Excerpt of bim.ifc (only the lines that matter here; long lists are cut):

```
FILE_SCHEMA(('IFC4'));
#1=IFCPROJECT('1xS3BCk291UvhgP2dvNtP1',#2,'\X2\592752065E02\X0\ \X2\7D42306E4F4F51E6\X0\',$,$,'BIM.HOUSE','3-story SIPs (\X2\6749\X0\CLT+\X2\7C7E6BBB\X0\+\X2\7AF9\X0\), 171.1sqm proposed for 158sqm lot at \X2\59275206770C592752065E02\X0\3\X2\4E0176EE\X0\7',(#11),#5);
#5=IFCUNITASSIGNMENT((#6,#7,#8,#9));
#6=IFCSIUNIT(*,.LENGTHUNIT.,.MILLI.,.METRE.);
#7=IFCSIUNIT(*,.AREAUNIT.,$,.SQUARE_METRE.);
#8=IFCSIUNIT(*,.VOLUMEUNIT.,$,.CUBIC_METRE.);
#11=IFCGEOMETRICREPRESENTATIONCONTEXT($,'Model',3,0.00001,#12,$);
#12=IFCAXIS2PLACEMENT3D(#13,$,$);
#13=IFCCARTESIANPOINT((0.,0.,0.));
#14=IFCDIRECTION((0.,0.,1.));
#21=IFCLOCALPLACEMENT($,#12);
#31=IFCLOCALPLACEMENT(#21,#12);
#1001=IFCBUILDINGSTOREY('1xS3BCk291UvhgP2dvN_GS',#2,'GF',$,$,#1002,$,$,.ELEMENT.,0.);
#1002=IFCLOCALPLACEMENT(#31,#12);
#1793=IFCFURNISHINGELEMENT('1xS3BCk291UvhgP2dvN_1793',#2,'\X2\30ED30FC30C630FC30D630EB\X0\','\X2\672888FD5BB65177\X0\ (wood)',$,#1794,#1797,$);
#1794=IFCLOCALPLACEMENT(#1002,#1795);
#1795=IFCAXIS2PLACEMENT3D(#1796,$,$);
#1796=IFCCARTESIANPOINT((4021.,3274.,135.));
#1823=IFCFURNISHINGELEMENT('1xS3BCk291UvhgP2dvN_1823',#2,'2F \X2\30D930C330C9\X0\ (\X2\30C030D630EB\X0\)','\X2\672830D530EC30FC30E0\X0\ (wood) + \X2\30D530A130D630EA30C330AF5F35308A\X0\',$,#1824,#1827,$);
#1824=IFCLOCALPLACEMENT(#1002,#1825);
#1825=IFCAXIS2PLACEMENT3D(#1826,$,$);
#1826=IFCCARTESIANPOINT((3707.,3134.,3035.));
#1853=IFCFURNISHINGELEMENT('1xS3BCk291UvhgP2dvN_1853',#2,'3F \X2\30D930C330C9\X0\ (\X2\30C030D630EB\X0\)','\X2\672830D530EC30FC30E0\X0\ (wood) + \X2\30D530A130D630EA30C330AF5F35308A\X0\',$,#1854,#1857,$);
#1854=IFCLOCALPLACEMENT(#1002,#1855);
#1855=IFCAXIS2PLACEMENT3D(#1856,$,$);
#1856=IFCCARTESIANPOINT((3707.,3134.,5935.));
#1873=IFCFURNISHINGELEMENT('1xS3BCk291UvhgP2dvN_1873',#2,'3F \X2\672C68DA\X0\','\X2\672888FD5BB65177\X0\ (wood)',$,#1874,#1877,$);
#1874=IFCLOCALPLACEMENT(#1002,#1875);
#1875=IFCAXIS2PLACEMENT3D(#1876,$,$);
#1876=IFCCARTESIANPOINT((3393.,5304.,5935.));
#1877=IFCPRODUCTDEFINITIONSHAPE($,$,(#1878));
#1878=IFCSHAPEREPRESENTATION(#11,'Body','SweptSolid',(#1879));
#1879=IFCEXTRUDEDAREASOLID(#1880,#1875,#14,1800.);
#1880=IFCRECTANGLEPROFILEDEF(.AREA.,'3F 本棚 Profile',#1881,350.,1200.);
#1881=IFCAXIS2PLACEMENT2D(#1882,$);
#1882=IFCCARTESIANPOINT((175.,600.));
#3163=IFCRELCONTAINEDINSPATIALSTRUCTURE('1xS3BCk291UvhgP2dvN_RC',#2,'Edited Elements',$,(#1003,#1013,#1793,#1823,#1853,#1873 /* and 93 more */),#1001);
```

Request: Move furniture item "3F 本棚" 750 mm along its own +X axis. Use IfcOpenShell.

```python
import ifcopenshell
import ifcopenshell.api.geometry
import ifcopenshell.util.placement

model = ifcopenshell.open("bim.ifc")

item = model.by_guid("1xS3BCk291UvhgP2dvN_1873")
matrix = ifcopenshell.util.placement.get_local_placement(item.ObjectPlacement)
matrix[:3, 3] += matrix[:3, 0] * 750.0
ifcopenshell.api.geometry.edit_object_placement(model, product=item, matrix=matrix, is_si=False)

print(ifcopenshell.util.placement.get_local_placement(item.ObjectPlacement).round(3) + 0.0)

model.write("bim-out.ifc")
```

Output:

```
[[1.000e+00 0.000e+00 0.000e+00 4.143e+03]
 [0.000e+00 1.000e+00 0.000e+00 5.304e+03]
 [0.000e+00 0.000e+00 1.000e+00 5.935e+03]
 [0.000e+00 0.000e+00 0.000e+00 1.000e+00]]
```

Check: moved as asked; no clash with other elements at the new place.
